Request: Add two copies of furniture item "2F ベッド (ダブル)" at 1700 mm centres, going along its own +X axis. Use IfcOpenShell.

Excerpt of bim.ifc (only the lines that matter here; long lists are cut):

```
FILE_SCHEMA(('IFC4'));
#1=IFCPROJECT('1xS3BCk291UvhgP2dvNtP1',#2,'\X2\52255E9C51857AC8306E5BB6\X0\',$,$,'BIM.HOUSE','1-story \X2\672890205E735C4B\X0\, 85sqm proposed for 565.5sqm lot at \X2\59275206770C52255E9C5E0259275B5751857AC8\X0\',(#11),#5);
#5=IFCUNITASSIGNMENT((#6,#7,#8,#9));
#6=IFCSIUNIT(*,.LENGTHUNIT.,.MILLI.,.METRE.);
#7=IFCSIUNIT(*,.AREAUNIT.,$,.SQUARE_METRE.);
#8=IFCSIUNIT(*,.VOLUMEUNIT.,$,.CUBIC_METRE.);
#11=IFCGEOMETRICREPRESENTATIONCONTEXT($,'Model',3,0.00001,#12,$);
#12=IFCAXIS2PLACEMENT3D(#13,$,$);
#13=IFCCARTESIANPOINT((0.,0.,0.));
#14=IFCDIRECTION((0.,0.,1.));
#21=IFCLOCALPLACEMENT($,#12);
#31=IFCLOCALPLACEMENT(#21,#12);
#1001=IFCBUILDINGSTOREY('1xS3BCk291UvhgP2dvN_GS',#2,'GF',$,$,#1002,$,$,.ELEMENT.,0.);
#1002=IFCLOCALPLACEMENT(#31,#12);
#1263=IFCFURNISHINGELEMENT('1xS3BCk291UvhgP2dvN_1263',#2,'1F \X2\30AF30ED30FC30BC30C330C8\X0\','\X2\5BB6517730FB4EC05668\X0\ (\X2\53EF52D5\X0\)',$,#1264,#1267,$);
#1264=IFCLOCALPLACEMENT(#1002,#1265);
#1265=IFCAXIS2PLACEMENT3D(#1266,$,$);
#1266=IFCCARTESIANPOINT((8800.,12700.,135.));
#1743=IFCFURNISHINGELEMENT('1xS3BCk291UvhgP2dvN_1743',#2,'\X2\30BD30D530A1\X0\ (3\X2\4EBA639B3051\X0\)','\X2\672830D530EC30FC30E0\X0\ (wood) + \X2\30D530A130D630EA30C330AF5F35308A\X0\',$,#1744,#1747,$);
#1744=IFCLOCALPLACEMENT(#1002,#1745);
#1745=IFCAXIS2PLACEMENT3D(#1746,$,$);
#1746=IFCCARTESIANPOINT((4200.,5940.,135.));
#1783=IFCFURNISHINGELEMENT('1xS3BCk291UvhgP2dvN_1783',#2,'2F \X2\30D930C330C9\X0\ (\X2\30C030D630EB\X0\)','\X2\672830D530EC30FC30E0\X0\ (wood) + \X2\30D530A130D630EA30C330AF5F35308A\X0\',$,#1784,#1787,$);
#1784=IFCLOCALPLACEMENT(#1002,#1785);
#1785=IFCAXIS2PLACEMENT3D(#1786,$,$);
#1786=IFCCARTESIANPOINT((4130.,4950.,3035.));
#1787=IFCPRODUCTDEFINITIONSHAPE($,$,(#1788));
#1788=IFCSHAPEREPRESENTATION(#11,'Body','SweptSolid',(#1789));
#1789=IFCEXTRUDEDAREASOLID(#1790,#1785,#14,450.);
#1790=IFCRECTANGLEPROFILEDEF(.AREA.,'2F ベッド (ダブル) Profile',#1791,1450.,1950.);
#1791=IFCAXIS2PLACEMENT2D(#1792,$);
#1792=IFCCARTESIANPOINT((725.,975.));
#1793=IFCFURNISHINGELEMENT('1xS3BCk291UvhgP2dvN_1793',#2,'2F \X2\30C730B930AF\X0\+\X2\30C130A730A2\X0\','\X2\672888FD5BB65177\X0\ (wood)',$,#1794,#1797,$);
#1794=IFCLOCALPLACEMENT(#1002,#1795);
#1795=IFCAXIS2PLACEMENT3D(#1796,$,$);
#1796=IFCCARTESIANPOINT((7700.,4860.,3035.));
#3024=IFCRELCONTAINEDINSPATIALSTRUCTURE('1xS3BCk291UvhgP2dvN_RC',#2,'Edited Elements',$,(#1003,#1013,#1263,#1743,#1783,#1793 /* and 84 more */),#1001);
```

```python
import ifcopenshell
import ifcopenshell.api.geometry
import ifcopenshell.api.root
import ifcopenshell.util.element
import ifcopenshell.util.placement
import ifcopenshell.util.unit

model = ifcopenshell.open("bim.ifc")
unit_scale = ifcopenshell.util.unit.calculate_unit_scale(model)


def reuse_history(source, copy):
    """copy_class also copies each property set's owner history, people and application; keep the originals."""
    for rel in copy.IsDefinedBy:
        if rel.is_a("IfcRelDefinesByProperties") and (history := rel.RelatingPropertyDefinition.OwnerHistory):
            rel.RelatingPropertyDefinition.OwnerHistory = source.OwnerHistory
            ifcopenshell.util.element.remove_deep2(model, history)


source = model.by_guid("1xS3BCk291UvhgP2dvN_1783")
base = ifcopenshell.util.placement.get_local_placement(source.ObjectPlacement)
step = base[:3, 0] * 1.7 / unit_scale

for i in range(1, 3):
    copy = ifcopenshell.api.root.copy_class(model, product=source)
    copy.Representation = ifcopenshell.util.element.copy_deep(
        model, source.Representation, exclude=["IfcGeometricRepresentationContext", "IfcRepresentationMap"]
    )
    reuse_history(source, copy)
    matrix = base.copy()
    matrix[:3, 3] += i * step
    print("added at", matrix[:3, 3].round(3) + 0.0)
    ifcopenshell.api.geometry.edit_object_placement(model, product=copy, matrix=matrix, is_si=False)

model.write("bim_updated.ifc")
```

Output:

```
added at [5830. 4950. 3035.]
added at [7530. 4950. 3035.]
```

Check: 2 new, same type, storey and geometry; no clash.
